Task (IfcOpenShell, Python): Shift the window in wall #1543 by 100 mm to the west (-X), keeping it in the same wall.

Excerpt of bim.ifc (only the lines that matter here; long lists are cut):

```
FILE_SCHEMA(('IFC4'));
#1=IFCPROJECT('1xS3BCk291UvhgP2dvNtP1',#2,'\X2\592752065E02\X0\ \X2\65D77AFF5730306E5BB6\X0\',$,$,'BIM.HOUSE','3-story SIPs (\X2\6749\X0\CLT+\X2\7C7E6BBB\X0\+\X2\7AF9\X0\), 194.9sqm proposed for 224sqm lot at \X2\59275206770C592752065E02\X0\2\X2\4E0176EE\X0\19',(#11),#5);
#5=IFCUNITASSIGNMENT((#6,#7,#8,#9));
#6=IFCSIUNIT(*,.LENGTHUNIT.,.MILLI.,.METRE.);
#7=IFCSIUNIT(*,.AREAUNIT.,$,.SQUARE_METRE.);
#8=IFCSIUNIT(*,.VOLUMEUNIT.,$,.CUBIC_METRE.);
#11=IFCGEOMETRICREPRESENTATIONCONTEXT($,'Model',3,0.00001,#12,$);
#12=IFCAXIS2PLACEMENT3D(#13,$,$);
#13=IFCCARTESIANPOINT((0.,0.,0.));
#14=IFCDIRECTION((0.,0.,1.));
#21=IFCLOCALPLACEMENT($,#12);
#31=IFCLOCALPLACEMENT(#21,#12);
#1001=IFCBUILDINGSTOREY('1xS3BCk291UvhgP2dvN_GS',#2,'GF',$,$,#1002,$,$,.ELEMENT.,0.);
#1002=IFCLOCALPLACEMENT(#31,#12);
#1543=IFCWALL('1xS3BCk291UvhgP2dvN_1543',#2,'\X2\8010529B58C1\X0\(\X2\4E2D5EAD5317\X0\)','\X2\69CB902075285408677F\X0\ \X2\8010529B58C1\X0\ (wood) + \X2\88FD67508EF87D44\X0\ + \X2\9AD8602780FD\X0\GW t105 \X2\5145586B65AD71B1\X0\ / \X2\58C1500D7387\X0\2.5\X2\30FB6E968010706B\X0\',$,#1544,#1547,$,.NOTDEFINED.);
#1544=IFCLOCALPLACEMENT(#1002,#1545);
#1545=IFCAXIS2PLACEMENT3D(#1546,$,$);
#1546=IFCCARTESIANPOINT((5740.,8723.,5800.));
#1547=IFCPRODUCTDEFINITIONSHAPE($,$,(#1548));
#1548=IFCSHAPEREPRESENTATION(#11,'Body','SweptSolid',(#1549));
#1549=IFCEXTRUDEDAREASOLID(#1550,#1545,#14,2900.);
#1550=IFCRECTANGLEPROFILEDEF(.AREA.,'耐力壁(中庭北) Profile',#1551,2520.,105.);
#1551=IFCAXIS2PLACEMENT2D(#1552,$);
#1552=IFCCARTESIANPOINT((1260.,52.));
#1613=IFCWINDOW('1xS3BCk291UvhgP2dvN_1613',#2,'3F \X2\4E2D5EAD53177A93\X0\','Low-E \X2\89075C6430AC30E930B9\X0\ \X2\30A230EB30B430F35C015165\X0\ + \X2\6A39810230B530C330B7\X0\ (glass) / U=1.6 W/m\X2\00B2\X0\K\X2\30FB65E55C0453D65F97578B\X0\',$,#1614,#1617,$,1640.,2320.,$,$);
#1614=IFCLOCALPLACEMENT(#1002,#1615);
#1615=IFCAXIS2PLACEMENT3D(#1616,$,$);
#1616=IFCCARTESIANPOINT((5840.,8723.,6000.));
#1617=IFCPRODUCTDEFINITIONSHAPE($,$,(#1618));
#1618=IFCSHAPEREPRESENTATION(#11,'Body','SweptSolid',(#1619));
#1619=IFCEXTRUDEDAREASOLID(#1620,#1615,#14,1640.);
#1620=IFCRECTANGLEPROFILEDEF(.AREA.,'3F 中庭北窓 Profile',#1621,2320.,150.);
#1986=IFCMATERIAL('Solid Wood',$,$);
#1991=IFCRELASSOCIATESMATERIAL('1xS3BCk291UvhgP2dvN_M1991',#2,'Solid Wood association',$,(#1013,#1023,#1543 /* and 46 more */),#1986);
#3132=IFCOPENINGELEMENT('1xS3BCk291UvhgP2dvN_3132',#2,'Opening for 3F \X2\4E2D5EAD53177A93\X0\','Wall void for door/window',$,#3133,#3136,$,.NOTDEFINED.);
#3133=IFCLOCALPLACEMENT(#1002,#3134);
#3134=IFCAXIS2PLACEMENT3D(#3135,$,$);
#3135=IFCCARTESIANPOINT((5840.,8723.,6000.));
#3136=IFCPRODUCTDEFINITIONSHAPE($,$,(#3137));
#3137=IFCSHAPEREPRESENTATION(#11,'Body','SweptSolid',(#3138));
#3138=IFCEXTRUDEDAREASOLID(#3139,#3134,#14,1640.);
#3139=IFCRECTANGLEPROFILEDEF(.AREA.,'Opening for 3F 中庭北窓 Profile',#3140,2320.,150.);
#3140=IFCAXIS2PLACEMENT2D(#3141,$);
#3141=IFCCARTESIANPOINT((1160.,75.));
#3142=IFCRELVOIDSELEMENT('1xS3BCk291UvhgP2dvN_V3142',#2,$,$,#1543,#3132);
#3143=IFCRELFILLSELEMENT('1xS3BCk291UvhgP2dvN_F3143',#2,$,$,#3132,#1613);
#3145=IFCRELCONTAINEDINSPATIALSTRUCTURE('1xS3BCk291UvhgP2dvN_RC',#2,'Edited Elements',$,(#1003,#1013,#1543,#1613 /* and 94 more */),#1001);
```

```python
import ifcopenshell
import ifcopenshell.api.geometry
import ifcopenshell.util.placement
import ifcopenshell.util.unit

model = ifcopenshell.open("bim.ifc")
unit_scale = ifcopenshell.util.unit.calculate_unit_scale(model)

window = model.by_guid("1xS3BCk291UvhgP2dvN_1613")
opening = window.FillsVoids[0].RelatingOpeningElement
wall = opening.VoidsElements[0].RelatingBuildingElement

wall_matrix = ifcopenshell.util.placement.get_local_placement(wall.ObjectPlacement)
shift = wall_matrix[:3, 0] * -0.1 / unit_scale
before = ifcopenshell.util.placement.get_local_placement(window.ObjectPlacement)[:3, 3].copy()

# The window is not placed relative to its opening, so move both.
for product in (opening, window):
    matrix = ifcopenshell.util.placement.get_local_placement(product.ObjectPlacement)
    matrix[:3, 3] += shift
    ifcopenshell.api.geometry.edit_object_placement(model, product=product, matrix=matrix, is_si=False)

after = ifcopenshell.util.placement.get_local_placement(window.ObjectPlacement)[:3, 3]
print("window moved by", (after - before).round(3) + 0.0)

model.write("bim_updated.ifc")
```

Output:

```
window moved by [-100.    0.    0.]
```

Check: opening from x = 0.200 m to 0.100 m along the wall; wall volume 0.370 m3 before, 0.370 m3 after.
